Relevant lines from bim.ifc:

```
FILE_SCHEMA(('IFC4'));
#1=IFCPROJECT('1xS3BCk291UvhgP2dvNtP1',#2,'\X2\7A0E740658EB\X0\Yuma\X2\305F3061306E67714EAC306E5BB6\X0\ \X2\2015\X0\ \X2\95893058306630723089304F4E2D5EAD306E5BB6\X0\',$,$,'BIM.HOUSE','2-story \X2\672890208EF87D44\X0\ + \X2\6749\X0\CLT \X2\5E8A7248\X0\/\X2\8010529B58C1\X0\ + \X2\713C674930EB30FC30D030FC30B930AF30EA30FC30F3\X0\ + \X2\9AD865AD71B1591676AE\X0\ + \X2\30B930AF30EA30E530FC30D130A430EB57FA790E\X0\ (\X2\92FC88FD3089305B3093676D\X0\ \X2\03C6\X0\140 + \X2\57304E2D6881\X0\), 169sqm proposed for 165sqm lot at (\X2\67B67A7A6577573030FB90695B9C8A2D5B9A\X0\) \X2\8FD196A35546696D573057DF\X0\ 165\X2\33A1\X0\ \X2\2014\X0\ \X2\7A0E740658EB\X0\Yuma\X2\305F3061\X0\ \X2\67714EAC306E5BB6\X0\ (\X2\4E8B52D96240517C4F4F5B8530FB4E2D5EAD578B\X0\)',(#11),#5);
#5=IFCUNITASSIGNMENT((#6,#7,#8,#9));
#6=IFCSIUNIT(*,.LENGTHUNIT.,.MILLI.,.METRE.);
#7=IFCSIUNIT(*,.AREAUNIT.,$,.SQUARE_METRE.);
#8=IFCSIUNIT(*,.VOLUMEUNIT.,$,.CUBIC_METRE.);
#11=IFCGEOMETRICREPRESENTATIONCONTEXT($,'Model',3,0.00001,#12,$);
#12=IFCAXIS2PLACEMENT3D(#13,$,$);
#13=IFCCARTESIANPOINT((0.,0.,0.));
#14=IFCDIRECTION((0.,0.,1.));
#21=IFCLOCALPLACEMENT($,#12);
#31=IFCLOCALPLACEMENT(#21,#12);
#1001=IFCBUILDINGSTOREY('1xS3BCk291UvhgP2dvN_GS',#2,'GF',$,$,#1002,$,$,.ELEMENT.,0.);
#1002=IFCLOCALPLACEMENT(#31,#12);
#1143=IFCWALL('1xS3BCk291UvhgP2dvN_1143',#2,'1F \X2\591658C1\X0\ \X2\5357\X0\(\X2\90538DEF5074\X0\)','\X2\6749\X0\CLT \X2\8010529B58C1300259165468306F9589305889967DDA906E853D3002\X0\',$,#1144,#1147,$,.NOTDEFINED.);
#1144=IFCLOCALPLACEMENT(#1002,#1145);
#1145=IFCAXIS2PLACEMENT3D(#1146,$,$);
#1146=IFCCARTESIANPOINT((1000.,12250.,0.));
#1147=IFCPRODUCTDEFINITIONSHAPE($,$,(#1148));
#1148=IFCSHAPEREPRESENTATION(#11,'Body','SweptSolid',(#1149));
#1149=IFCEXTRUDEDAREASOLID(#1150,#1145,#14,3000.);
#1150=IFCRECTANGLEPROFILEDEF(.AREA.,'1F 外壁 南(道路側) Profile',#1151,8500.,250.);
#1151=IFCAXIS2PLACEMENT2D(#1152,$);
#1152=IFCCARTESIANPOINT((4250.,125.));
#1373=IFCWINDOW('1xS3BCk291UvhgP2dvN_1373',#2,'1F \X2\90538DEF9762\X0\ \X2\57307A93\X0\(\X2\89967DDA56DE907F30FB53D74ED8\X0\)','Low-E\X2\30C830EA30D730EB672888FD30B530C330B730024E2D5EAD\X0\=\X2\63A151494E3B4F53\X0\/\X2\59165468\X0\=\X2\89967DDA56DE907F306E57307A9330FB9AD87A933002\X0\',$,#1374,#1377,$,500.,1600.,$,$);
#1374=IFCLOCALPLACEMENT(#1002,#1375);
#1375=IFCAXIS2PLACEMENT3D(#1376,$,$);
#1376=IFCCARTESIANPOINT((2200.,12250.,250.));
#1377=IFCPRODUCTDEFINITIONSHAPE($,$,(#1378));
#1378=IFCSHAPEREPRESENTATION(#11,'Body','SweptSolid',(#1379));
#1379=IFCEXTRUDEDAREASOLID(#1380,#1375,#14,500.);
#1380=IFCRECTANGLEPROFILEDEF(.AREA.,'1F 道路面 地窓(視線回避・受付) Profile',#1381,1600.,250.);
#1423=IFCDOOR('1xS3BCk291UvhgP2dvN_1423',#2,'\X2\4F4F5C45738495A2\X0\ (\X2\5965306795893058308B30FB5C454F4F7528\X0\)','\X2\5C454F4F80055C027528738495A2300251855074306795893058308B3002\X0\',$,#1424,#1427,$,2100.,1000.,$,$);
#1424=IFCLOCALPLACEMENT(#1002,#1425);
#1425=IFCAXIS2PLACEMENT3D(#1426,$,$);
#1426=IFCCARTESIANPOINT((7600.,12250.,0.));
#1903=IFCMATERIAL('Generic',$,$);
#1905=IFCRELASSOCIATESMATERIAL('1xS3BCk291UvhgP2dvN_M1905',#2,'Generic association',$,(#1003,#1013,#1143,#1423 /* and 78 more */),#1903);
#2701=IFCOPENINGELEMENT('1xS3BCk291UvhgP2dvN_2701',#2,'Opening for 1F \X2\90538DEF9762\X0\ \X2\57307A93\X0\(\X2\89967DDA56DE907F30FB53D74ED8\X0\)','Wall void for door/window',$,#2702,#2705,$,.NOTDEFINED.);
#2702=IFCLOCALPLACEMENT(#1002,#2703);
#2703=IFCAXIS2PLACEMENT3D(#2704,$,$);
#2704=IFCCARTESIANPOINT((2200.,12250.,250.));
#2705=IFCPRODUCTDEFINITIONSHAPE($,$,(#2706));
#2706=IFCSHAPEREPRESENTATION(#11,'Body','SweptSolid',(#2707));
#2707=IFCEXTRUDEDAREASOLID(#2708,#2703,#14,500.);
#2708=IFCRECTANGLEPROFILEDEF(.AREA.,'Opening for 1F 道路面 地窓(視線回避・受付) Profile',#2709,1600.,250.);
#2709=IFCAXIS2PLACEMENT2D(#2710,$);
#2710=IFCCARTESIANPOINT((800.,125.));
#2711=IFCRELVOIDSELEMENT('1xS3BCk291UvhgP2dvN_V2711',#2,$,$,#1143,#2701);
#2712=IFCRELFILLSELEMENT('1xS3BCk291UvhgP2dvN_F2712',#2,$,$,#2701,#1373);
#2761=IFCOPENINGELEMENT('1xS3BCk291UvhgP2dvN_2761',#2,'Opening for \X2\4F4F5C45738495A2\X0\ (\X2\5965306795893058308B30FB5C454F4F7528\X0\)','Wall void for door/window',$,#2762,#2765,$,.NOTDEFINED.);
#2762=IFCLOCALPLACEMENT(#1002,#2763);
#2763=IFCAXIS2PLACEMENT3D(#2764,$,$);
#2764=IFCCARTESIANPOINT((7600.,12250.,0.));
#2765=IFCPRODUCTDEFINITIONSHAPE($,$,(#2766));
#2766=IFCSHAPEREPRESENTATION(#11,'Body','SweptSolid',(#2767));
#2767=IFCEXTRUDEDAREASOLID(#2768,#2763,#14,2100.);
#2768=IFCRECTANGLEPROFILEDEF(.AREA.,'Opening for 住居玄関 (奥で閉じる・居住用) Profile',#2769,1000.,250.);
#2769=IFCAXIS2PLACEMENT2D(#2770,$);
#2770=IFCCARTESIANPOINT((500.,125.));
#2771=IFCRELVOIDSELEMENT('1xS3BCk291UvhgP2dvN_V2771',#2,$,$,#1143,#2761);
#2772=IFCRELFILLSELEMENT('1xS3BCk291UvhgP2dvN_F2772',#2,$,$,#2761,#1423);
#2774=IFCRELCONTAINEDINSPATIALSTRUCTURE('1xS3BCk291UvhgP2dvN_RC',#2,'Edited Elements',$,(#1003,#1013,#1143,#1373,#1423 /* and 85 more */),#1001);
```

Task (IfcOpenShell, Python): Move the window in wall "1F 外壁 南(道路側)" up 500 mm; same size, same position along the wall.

```python
import numpy as np
import ifcopenshell
import ifcopenshell.api.geometry
import ifcopenshell.util.placement
import ifcopenshell.util.unit

model = ifcopenshell.open("bim.ifc")
unit_scale = ifcopenshell.util.unit.calculate_unit_scale(model)

window = model.by_id(1373)
opening = window.FillsVoids[0].RelatingOpeningElement
dz = 0.5 / unit_scale

shift = np.array([0.0, 0.0, dz])
# The window is not placed relative to its opening, so move both.
for product in (opening, window):
    matrix = ifcopenshell.util.placement.get_local_placement(product.ObjectPlacement)
    matrix[:3, 3] += shift
    ifcopenshell.api.geometry.edit_object_placement(model, product=product, matrix=matrix, is_si=False)

print(f"moved by {dz * unit_scale:+.3f} m")

model.write("bim-out.ifc")
```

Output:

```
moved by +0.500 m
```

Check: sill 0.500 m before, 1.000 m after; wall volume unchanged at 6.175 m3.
